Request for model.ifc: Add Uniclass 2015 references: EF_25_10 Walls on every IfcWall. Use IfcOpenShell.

First a look at what the model holds.

```python
import ifcopenshell

model = ifcopenshell.open("model.ifc")
print(model.schema)
print("classifications:", [c.Name for c in model.by_type("IfcClassification")])
for ifc_class in ("IfcDoor", "IfcRoof", "IfcStair", "IfcWall", "IfcWindow"):
    print(ifc_class, len(model.by_type(ifc_class)))
```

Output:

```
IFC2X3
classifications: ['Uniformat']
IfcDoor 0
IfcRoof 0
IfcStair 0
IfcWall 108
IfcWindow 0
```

```python
import ifcopenshell
import ifcopenshell.api.classification

model = ifcopenshell.open("model.ifc")

# IFC2X3 requires Source and Edition and has no link from the project to the system.
system = model.create_entity("IfcClassification", Source="NBS", Edition="2015", Name="Uniclass 2015")

codes = {
    "IfcWall": ("EF_25_10", "Walls"),
}
for ifc_class, (code, name) in codes.items():
    products = model.by_type(ifc_class)
    ifcopenshell.api.classification.add_reference(
        model, products=products, classification=system, identification=code, name=name
    )
    print(code, len(products))

model.write("model_edited.ifc")
```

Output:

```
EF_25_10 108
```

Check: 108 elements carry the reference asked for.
